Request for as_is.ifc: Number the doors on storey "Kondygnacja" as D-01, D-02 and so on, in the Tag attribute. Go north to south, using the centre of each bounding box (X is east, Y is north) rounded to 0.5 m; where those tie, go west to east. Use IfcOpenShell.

First a look at what the model holds.

```python
import ifcopenshell
import ifcopenshell.util.element
import ifcopenshell.util.placement

model = ifcopenshell.open("as_is.ifc")
print(model.schema)
storey = next(s for s in model.by_type("IfcBuildingStorey") if s.Name == "Kondygnacja")
doors = [e for e in ifcopenshell.util.element.get_decomposition(storey) if e.is_a("IfcDoor")]
for e in sorted(doors, key=lambda e: e.id()):
    origin = ifcopenshell.util.placement.get_local_placement(e.ObjectPlacement)[:3, 3]
    print(e.id(), e.Tag, e.Name, origin.round(2) + 0.0, sep=" | ")
```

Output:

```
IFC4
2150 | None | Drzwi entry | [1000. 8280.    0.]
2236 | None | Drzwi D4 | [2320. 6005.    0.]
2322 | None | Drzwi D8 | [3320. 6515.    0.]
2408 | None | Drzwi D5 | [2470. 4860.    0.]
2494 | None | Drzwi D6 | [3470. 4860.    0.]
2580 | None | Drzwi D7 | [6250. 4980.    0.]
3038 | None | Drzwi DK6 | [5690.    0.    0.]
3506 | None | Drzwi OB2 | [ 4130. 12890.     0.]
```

```python
import ifcopenshell
import ifcopenshell.geom
import ifcopenshell.util.element
import ifcopenshell.util.shape

model = ifcopenshell.open("as_is.ifc")
settings = ifcopenshell.geom.settings()
settings.set("use-world-coords", True)


def centre(element):
    shape = ifcopenshell.geom.create_shape(settings, element)
    return ifcopenshell.util.shape.get_bbox_centroid(shape.geometry)


storey = next(s for s in model.by_type("IfcBuildingStorey") if s.Name == "Kondygnacja")
doors = [e for e in ifcopenshell.util.element.get_decomposition(storey) if e.is_a("IfcDoor")]

# Insertion points can sit at a corner or the storey origin, so sort by the geometry (in metres).
centres = {e: centre(e) for e in doors}
doors.sort(key=lambda e: (-round(centres[e][1] / 0.5), centres[e][0]))

for i, e in enumerate(doors, start=1):
    number = f"D-{i:02d}"
    e.Tag = number
    print(e.id(), number)

model.write("as_is_rev.ifc")
```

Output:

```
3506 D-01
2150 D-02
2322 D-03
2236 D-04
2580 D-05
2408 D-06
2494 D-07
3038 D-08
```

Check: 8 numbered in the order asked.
